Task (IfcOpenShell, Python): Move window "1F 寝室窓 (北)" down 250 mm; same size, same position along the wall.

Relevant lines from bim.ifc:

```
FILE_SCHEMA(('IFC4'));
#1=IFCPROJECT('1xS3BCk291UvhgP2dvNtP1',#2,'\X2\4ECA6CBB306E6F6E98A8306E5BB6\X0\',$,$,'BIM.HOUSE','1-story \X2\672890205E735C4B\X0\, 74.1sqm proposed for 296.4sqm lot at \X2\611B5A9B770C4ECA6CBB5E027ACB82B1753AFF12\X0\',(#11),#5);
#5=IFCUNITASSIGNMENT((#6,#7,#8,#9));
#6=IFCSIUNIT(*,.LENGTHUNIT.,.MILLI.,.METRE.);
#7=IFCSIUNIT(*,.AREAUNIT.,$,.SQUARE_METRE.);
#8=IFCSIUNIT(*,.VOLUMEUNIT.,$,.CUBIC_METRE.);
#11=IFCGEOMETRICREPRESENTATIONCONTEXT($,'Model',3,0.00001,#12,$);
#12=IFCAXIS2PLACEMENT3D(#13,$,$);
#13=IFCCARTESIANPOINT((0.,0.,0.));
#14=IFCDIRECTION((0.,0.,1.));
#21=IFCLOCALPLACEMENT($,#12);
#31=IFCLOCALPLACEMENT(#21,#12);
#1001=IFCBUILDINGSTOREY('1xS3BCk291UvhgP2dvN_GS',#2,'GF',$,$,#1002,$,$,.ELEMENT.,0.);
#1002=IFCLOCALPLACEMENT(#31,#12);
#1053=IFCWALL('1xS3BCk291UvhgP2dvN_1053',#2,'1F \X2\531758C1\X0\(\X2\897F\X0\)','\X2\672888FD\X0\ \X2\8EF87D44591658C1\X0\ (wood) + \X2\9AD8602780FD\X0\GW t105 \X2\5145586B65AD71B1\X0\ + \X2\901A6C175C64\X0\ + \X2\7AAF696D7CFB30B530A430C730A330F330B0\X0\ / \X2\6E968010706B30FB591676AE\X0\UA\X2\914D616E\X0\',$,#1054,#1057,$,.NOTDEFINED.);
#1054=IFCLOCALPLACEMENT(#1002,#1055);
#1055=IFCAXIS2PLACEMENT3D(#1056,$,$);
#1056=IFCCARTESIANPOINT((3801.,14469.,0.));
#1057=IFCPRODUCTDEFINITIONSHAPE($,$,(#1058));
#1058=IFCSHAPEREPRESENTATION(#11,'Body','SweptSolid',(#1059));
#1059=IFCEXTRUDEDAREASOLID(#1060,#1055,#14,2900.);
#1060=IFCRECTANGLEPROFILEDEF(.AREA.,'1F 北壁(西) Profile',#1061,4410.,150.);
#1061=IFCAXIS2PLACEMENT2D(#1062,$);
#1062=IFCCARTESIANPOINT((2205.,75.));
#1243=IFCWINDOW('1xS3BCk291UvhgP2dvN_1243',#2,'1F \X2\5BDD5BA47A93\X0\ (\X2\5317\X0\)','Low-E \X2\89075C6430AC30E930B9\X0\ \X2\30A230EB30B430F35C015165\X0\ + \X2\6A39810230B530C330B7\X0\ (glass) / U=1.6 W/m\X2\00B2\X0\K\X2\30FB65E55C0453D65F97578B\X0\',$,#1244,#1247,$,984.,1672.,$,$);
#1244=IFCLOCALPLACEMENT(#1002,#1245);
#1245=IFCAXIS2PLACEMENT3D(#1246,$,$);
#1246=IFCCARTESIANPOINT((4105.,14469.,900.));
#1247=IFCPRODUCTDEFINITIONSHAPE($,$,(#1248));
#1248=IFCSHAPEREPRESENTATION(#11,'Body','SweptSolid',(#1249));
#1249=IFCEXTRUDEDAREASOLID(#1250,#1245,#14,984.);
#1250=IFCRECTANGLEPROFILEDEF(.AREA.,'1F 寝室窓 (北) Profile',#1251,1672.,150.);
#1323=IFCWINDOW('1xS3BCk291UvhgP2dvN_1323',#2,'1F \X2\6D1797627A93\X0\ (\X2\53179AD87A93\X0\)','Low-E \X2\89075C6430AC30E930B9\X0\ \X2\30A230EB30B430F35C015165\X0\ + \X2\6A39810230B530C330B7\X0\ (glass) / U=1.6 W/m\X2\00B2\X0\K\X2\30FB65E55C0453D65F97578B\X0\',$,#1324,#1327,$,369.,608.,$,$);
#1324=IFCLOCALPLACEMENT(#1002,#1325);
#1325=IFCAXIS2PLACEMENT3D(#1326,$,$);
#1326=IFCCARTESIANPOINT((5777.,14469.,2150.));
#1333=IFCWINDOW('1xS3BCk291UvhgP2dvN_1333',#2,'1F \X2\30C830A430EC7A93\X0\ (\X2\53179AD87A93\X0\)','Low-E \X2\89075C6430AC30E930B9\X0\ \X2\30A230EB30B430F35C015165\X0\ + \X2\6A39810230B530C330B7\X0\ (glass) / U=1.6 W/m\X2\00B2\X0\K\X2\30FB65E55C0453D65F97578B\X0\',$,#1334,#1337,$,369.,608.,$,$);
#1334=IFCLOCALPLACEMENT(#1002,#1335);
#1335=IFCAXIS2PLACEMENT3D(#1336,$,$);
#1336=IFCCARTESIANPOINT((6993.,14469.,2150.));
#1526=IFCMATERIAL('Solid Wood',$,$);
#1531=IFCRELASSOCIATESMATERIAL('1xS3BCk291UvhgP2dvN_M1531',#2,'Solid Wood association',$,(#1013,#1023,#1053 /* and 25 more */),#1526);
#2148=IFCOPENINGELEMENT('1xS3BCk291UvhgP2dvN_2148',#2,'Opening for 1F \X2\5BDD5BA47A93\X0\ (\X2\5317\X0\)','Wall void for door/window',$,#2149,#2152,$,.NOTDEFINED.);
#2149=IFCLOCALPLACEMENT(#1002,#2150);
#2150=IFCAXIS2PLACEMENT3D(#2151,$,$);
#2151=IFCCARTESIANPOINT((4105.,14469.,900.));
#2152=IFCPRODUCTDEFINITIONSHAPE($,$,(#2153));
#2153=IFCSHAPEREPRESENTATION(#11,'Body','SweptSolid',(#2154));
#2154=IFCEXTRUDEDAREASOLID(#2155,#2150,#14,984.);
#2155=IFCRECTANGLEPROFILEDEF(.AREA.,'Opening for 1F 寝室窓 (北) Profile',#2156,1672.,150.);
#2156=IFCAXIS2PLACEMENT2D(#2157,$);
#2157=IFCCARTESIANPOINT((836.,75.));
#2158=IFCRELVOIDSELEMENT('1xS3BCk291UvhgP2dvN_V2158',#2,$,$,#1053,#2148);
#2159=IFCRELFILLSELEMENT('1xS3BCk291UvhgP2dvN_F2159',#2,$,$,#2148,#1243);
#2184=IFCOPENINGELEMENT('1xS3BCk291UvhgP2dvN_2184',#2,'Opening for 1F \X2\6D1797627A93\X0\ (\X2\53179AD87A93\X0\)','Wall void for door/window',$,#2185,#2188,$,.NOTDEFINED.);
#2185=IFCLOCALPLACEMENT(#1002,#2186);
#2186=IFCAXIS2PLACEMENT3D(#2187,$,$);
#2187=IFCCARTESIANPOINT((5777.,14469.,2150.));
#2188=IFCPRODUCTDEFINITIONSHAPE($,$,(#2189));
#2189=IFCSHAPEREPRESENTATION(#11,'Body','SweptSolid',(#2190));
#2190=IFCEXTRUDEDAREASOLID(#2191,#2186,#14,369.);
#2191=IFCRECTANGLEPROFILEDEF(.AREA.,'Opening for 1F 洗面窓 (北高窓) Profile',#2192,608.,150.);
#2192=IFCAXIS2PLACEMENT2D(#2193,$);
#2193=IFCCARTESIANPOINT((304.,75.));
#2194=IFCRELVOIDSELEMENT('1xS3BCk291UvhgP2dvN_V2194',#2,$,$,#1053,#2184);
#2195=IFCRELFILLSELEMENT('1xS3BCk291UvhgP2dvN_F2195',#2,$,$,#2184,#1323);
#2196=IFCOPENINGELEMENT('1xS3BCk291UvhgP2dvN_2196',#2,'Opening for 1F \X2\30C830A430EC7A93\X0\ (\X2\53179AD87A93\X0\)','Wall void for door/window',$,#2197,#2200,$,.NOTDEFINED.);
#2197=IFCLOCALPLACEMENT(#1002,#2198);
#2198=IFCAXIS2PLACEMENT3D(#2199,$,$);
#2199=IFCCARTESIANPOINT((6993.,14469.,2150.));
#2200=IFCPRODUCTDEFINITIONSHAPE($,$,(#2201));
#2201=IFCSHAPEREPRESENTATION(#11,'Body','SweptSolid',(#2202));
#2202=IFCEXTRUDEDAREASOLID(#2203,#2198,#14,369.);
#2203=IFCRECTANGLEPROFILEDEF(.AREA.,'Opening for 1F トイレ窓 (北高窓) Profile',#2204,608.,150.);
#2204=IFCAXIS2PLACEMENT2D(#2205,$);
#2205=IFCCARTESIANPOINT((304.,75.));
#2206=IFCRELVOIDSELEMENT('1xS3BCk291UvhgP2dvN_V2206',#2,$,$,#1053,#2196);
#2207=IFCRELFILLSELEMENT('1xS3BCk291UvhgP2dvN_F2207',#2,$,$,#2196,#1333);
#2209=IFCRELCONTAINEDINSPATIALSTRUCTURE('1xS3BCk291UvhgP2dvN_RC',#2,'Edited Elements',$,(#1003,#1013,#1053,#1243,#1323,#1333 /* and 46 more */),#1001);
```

```python
import numpy as np
import ifcopenshell
import ifcopenshell.api.geometry
import ifcopenshell.util.placement
import ifcopenshell.util.unit

model = ifcopenshell.open("bim.ifc")
unit_scale = ifcopenshell.util.unit.calculate_unit_scale(model)

window = model.by_id(1243)
opening = window.FillsVoids[0].RelatingOpeningElement
dz = -250.0

shift = np.array([0.0, 0.0, dz])
# The window is not placed relative to its opening, so move both.
for product in (opening, window):
    matrix = ifcopenshell.util.placement.get_local_placement(product.ObjectPlacement)
    matrix[:3, 3] += shift
    ifcopenshell.api.geometry.edit_object_placement(model, product=product, matrix=matrix, is_si=False)

print(f"moved by {dz * unit_scale:+.3f} m")

model.write("bim-out.ifc")
```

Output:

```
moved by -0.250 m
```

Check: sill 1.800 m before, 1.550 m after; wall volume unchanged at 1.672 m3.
